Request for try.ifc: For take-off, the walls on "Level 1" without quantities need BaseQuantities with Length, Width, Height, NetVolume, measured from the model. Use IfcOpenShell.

First a look at what the model holds.

```python
import ifcopenshell
import ifcopenshell.util.element
import ifcopenshell.util.unit

model = ifcopenshell.open("try.ifc")
print(model.schema)
for unit_type in ("LENGTHUNIT", "AREAUNIT", "VOLUMEUNIT"):
    print(unit_type, ifcopenshell.util.unit.calculate_unit_scale(model, unit_type))
storey = next(s for s in model.by_type("IfcBuildingStorey") if s.Name == "Level 1")
walls = [e for e in ifcopenshell.util.element.get_decomposition(storey) if e.is_a("IfcWall")]
for e in sorted(walls, key=lambda e: e.id()):
    print(e.id(), e.is_a(), e.Name, list(ifcopenshell.util.element.get_psets(e, qtos_only=True)), sep=" | ")
```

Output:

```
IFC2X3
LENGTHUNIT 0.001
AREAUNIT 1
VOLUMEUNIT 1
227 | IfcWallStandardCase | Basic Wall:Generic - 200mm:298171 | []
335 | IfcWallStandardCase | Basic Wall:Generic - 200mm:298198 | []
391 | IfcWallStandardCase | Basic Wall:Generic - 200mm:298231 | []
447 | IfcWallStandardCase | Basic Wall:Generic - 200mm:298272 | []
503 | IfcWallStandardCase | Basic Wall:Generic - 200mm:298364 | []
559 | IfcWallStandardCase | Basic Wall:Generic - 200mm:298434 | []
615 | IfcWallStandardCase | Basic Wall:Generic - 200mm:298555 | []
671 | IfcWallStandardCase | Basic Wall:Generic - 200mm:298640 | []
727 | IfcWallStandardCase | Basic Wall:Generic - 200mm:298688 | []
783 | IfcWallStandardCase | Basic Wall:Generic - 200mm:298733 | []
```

```python
import ifcopenshell
import ifcopenshell.api.pset
import ifcopenshell.geom
import ifcopenshell.util.element
import ifcopenshell.util.shape
import ifcopenshell.util.unit

model = ifcopenshell.open("try.ifc")
unit_scale = ifcopenshell.util.unit.calculate_unit_scale(model)
volume_scale = ifcopenshell.util.unit.calculate_unit_scale(model, "VOLUMEUNIT")
settings = ifcopenshell.geom.settings()

storey = next(s for s in model.by_type("IfcBuildingStorey") if s.Name == "Level 1")
walls = [e for e in ifcopenshell.util.element.get_decomposition(storey) if e.is_a("IfcWall")]

for e in sorted(walls, key=lambda e: e.id()):
    if ifcopenshell.util.element.get_psets(e, qtos_only=True, should_inherit=False):
        continue
    # Geometry comes back in metres, in the element's own axes.
    shape = ifcopenshell.geom.create_shape(settings, e)
    values = {
        "Length": ifcopenshell.util.shape.get_x(shape.geometry) / unit_scale,
        "Width": ifcopenshell.util.shape.get_y(shape.geometry) / unit_scale,
        "Height": ifcopenshell.util.shape.get_z(shape.geometry) / unit_scale,
        "NetVolume": ifcopenshell.util.shape.get_volume(shape.geometry) / volume_scale,
    }
    qto = ifcopenshell.api.pset.add_qto(model, product=e, name="BaseQuantities")
    ifcopenshell.api.pset.edit_qto(model, qto=qto, properties=values)
    print(e.id(), {k: round(v, 3) for k, v in values.items()})

model.write("try-out.ifc")
```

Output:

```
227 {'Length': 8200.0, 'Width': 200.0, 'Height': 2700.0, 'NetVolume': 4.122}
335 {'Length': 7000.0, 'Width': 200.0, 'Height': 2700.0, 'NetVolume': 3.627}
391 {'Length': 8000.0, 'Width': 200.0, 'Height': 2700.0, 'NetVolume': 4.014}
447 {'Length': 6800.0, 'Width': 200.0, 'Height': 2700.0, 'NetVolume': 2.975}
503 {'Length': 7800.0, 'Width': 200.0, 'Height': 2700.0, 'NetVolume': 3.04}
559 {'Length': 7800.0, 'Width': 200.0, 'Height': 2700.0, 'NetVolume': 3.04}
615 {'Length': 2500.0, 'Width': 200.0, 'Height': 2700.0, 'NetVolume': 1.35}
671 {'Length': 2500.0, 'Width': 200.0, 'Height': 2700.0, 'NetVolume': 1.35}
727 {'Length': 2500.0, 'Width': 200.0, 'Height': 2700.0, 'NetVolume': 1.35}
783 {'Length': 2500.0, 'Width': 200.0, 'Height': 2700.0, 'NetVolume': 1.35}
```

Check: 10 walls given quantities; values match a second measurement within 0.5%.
